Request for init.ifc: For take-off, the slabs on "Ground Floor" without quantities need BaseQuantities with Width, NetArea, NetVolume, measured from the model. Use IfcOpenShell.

First a look at what the model holds.

```python
import ifcopenshell
import ifcopenshell.util.element
import ifcopenshell.util.unit

model = ifcopenshell.open("init.ifc")
print(model.schema)
for unit_type in ("LENGTHUNIT", "AREAUNIT", "VOLUMEUNIT"):
    print(unit_type, ifcopenshell.util.unit.calculate_unit_scale(model, unit_type))
storey = next(s for s in model.by_type("IfcBuildingStorey") if s.Name == "Ground Floor")
slabs = [e for e in ifcopenshell.util.element.get_decomposition(storey) if e.is_a("IfcSlab")]
for e in sorted(slabs, key=lambda e: e.id()):
    print(e.id(), e.is_a(), e.Name, list(ifcopenshell.util.element.get_psets(e, qtos_only=True)), sep=" | ")
```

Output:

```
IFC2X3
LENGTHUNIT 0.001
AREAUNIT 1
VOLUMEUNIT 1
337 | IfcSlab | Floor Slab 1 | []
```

```python
import ifcopenshell
import ifcopenshell.api.pset
import ifcopenshell.geom
import ifcopenshell.util.element
import ifcopenshell.util.shape
import ifcopenshell.util.unit

model = ifcopenshell.open("init.ifc")
unit_scale = ifcopenshell.util.unit.calculate_unit_scale(model)
area_scale = ifcopenshell.util.unit.calculate_unit_scale(model, "AREAUNIT")
volume_scale = ifcopenshell.util.unit.calculate_unit_scale(model, "VOLUMEUNIT")
settings = ifcopenshell.geom.settings()

storey = next(s for s in model.by_type("IfcBuildingStorey") if s.Name == "Ground Floor")
slabs = [e for e in ifcopenshell.util.element.get_decomposition(storey) if e.is_a("IfcSlab")]

for e in sorted(slabs, key=lambda e: e.id()):
    if ifcopenshell.util.element.get_psets(e, qtos_only=True, should_inherit=False):
        continue
    # Geometry comes back in metres, in the element's own axes.
    shape = ifcopenshell.geom.create_shape(settings, e)
    values = {
        "Width": ifcopenshell.util.shape.get_z(shape.geometry) / unit_scale,
        "NetArea": ifcopenshell.util.shape.get_footprint_area(shape.geometry) / area_scale,
        "NetVolume": ifcopenshell.util.shape.get_volume(shape.geometry) / volume_scale,
    }
    qto = ifcopenshell.api.pset.add_qto(model, product=e, name="BaseQuantities")
    ifcopenshell.api.pset.edit_qto(model, qto=qto, properties=values)
    print(e.id(), {k: round(v, 3) for k, v in values.items()})

model.write("init_rev.ifc")
```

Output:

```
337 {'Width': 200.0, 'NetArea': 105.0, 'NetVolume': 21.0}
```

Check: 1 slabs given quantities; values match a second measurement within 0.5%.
